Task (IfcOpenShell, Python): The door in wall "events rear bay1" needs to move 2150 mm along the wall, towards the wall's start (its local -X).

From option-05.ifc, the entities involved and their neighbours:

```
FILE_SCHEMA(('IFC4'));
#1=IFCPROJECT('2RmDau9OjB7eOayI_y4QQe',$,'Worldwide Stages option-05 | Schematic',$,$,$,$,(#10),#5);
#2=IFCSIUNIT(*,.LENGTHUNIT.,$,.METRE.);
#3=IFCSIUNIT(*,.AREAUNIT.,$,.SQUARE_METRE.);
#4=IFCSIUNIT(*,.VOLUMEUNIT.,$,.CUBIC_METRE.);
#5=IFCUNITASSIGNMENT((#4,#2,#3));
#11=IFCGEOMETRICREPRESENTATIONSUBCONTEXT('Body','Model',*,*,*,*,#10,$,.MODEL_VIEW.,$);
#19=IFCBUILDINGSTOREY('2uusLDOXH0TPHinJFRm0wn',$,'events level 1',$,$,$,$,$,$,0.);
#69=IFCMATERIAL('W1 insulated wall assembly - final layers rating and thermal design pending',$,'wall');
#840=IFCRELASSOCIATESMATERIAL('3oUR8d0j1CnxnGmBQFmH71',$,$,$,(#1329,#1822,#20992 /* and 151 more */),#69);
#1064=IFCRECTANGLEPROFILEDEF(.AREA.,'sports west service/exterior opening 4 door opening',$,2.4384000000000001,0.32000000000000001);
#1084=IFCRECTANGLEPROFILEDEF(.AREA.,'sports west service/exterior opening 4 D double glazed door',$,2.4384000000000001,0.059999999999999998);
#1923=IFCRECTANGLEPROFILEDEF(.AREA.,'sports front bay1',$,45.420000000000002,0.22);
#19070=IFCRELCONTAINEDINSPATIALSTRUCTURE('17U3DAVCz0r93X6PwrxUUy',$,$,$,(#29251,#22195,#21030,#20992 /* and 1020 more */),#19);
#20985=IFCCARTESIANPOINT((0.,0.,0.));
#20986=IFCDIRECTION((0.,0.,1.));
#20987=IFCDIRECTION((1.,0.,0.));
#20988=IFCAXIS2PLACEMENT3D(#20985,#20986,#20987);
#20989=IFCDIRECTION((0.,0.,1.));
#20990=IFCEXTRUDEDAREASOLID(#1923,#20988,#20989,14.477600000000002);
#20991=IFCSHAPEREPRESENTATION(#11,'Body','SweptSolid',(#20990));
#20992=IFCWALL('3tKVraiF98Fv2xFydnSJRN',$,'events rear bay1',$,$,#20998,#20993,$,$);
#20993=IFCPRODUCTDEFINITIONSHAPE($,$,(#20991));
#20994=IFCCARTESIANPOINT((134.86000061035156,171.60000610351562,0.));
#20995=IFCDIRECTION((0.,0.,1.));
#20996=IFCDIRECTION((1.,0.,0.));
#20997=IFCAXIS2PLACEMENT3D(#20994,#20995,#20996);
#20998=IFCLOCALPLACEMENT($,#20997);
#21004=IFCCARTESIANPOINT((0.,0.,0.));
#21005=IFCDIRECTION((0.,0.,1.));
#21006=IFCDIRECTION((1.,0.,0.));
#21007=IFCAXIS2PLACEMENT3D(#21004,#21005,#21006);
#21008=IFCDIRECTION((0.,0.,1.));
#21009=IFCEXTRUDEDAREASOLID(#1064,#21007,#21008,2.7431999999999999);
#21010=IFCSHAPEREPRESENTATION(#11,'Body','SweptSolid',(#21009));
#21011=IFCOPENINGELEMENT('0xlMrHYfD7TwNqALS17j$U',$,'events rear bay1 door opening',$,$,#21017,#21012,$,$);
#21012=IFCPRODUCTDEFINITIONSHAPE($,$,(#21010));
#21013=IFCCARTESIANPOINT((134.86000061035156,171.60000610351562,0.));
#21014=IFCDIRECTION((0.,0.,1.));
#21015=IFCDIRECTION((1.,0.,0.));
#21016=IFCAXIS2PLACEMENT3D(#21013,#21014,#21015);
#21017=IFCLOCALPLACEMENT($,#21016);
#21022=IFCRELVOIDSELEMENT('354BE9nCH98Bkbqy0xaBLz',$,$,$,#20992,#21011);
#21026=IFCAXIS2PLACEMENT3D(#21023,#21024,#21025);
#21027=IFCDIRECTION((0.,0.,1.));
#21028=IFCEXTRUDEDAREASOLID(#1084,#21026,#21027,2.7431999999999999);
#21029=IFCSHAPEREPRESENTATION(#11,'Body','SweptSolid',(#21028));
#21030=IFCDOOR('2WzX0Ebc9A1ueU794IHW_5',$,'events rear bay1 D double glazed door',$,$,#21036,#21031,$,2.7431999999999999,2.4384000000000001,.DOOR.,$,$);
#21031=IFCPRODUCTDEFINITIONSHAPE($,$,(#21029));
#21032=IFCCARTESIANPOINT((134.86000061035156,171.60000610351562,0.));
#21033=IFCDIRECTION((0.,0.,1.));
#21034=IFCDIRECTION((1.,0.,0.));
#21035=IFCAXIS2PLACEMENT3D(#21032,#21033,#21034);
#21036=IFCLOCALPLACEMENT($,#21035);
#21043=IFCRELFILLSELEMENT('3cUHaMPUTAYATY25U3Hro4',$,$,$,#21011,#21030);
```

```python
import ifcopenshell
import ifcopenshell.api.geometry
import ifcopenshell.util.placement

model = ifcopenshell.open("option-05.ifc")

door = model.by_id(21030)
opening = door.FillsVoids[0].RelatingOpeningElement
wall = opening.VoidsElements[0].RelatingBuildingElement

wall_matrix = ifcopenshell.util.placement.get_local_placement(wall.ObjectPlacement)
shift = wall_matrix[:3, 0] * -2.15
before = ifcopenshell.util.placement.get_local_placement(door.ObjectPlacement)[:3, 3].copy()

# The door is not placed relative to its opening, so move both.
for product in (opening, door):
    matrix = ifcopenshell.util.placement.get_local_placement(product.ObjectPlacement)
    matrix[:3, 3] += shift
    ifcopenshell.api.geometry.edit_object_placement(model, product=product, matrix=matrix, is_si=False)

after = ifcopenshell.util.placement.get_local_placement(door.ObjectPlacement)[:3, 3]
print("door moved by", (after - before).round(3) + 0.0)

model.write("option-05_rev.ifc")
```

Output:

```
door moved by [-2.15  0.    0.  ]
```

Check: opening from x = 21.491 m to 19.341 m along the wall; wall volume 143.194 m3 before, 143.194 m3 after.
